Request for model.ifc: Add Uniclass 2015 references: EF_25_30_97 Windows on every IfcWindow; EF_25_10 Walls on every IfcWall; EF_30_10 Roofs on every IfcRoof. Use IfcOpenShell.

First a look at what the model holds.

```python
import ifcopenshell

model = ifcopenshell.open("model.ifc")
print(model.schema)
print("classifications:", [c.Name for c in model.by_type("IfcClassification")])
for ifc_class in ("IfcDoor", "IfcRoof", "IfcStair", "IfcWall", "IfcWindow"):
    print(ifc_class, len(model.by_type(ifc_class)))
```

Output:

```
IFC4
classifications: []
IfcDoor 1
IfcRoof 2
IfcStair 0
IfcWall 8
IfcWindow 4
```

```python
import ifcopenshell
import ifcopenshell.api.classification

model = ifcopenshell.open("model.ifc")

system = ifcopenshell.api.classification.add_classification(model, classification="Uniclass 2015")

codes = {
    "IfcWindow": ("EF_25_30_97", "Windows"),
    "IfcWall": ("EF_25_10", "Walls"),
    "IfcRoof": ("EF_30_10", "Roofs"),
}
for ifc_class, (code, name) in codes.items():
    products = model.by_type(ifc_class)
    ifcopenshell.api.classification.add_reference(
        model, products=products, classification=system, identification=code, name=name
    )
    print(code, len(products))

model.write("model_v2.ifc")
```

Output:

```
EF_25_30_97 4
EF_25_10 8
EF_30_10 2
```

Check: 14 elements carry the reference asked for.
